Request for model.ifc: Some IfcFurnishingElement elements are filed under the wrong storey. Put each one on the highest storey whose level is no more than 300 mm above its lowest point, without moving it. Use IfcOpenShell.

First a look at what the model holds.

```python
import ifcopenshell
import ifcopenshell.util.element
import ifcopenshell.util.placement

model = ifcopenshell.open("model.ifc")
print(model.schema)
for storey in model.by_type("IfcBuildingStorey"):
    level = ifcopenshell.util.placement.get_storey_elevation(storey)
    count = sum(e.is_a("IfcFurnishingElement") for e in ifcopenshell.util.element.get_contained(storey))
    print(storey.id(), storey.Name, round(level, 3), count, sep=" | ")
```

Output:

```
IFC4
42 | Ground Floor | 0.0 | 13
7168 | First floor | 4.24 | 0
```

```python
import ifcopenshell
import ifcopenshell.api.spatial
import ifcopenshell.geom
import ifcopenshell.util.element
import ifcopenshell.util.placement
import ifcopenshell.util.shape
import ifcopenshell.util.unit

model = ifcopenshell.open("model.ifc")
unit_scale = ifcopenshell.util.unit.calculate_unit_scale(model)
settings = ifcopenshell.geom.settings()

levels = sorted(
    ((ifcopenshell.util.placement.get_storey_elevation(s) * unit_scale, s) for s in model.by_type("IfcBuildingStorey")),
    key=lambda pair: pair[0],
)

for e in model.by_type("IfcFurnishingElement"):
    current = e.ContainedInStructure[0].RelatingStructure if e.ContainedInStructure else None
    if current is None or not current.is_a("IfcBuildingStorey"):
        continue
    shape = ifcopenshell.geom.create_shape(settings, e)
    bottom = ifcopenshell.util.shape.get_shape_bottom_elevation(shape, shape.geometry)
    below = [s for level, s in levels if level <= bottom + 0.3]
    storey = below[-1] if below else levels[0][1]
    if storey != current:
        # assign_container keeps the world position.
        ifcopenshell.api.spatial.assign_container(model, products=[e], relating_structure=storey)
        print(e.id(), current.Name, "->", storey.Name)

model.write("model_v2.ifc")
```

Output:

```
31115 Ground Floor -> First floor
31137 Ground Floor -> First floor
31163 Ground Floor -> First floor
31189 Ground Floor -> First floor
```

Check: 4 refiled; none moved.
